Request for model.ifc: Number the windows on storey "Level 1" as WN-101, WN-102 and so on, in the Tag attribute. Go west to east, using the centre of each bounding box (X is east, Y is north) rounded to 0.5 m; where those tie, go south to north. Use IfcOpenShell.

First a look at what the model holds.

```python
import ifcopenshell
import ifcopenshell.util.element
import ifcopenshell.util.placement

model = ifcopenshell.open("model.ifc")
print(model.schema)
storey = next(s for s in model.by_type("IfcBuildingStorey") if s.Name == "Level 1")
windows = [e for e in ifcopenshell.util.element.get_decomposition(storey) if e.is_a("IfcWindow")]
for e in sorted(windows, key=lambda e: e.id()):
    origin = ifcopenshell.util.placement.get_local_placement(e.ObjectPlacement)[:3, 3]
    print(e.id(), e.Tag, e.Name, origin.round(2) + 0.0, sep=" | ")
```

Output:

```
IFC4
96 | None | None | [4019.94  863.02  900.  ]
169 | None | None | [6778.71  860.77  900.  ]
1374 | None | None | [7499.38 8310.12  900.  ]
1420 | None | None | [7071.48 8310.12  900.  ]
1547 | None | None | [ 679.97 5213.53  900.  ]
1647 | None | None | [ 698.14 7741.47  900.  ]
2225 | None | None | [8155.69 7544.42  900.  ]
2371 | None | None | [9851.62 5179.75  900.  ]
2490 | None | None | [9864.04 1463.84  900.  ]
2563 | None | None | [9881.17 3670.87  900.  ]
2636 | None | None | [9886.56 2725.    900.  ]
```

```python
import ifcopenshell
import ifcopenshell.geom
import ifcopenshell.util.element
import ifcopenshell.util.shape

model = ifcopenshell.open("model.ifc")
settings = ifcopenshell.geom.settings()
settings.set("use-world-coords", True)


def centre(element):
    shape = ifcopenshell.geom.create_shape(settings, element)
    return ifcopenshell.util.shape.get_bbox_centroid(shape.geometry)


storey = next(s for s in model.by_type("IfcBuildingStorey") if s.Name == "Level 1")
windows = [e for e in ifcopenshell.util.element.get_decomposition(storey) if e.is_a("IfcWindow")]

# Insertion points can sit at a corner or the storey origin, so sort by the geometry (in metres).
centres = {e: centre(e) for e in windows}
windows.sort(key=lambda e: (round(centres[e][0] / 0.5), centres[e][1]))

for i, e in enumerate(windows, start=1):
    number = f"WN-1{i:02d}"
    e.Tag = number
    print(e.id(), number)

model.write("model_updated.ifc")
```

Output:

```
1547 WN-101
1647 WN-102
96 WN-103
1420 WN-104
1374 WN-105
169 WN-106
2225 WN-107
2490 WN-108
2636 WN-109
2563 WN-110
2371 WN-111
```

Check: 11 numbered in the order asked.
